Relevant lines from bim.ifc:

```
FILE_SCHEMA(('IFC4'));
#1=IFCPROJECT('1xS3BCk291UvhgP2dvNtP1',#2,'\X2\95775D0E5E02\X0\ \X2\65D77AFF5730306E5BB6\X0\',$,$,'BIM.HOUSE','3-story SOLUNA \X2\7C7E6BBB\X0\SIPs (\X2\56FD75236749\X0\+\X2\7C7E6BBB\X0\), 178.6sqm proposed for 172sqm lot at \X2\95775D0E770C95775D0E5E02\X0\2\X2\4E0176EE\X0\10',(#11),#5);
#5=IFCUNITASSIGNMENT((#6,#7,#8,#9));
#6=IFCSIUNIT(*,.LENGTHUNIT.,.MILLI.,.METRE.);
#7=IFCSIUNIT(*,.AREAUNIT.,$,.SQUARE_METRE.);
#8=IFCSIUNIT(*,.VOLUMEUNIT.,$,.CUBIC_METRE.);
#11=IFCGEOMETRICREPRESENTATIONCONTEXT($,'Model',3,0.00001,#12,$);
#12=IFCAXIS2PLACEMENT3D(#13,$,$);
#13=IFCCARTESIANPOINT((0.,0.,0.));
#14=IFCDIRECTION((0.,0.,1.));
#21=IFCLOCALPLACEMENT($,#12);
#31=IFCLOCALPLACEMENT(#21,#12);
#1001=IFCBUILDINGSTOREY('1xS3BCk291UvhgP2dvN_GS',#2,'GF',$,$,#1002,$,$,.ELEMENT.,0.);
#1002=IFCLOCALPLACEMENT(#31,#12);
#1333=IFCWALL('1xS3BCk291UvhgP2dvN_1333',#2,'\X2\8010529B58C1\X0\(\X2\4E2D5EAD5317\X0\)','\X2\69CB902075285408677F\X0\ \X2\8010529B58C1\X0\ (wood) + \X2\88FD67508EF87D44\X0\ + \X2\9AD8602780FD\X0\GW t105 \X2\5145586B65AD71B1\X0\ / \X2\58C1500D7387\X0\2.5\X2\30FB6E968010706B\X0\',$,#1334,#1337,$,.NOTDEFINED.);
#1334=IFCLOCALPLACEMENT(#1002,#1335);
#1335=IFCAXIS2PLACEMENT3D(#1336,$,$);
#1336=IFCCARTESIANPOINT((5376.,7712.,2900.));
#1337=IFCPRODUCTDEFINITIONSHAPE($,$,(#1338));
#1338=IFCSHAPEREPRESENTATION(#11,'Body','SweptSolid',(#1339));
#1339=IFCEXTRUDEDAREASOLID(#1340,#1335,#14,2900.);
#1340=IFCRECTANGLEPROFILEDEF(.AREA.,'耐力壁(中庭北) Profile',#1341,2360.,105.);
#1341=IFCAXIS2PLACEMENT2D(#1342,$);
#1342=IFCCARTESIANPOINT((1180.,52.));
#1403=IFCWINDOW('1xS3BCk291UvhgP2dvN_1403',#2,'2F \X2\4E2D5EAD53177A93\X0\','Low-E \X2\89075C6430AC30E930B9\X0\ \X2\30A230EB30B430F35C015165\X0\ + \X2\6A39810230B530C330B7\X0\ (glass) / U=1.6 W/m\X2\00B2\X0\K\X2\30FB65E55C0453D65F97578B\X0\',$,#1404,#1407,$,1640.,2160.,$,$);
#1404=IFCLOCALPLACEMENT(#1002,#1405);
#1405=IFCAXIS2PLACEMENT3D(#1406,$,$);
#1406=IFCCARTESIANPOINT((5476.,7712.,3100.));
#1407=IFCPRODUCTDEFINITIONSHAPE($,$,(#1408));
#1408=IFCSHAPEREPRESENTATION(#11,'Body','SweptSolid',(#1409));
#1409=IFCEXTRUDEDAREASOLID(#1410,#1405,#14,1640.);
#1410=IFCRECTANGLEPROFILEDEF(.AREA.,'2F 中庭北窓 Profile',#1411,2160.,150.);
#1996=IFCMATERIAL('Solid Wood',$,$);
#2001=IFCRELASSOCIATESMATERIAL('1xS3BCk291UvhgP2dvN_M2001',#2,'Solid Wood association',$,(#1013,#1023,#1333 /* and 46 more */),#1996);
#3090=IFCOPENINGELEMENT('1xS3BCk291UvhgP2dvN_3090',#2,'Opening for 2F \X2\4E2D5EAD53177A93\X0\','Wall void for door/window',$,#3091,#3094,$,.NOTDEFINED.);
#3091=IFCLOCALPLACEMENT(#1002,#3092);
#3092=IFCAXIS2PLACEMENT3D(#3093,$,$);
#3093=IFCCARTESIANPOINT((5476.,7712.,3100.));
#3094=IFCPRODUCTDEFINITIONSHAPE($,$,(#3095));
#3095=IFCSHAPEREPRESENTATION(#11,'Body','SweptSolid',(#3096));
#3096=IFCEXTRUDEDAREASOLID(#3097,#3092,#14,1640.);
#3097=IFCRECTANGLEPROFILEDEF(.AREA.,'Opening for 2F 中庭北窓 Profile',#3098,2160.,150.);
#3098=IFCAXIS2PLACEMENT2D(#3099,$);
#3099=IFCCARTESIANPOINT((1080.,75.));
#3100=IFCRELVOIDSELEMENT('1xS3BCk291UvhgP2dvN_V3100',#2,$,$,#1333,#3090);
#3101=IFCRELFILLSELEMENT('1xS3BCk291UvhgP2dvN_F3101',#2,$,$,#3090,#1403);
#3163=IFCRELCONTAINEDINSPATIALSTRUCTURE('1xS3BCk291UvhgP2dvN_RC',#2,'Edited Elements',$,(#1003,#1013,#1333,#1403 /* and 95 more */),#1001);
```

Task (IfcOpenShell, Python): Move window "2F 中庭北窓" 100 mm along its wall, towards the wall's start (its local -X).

```python
import ifcopenshell
import ifcopenshell.api.geometry
import ifcopenshell.util.placement

model = ifcopenshell.open("bim.ifc")

window = model.by_guid("1xS3BCk291UvhgP2dvN_1403")
opening = window.FillsVoids[0].RelatingOpeningElement
wall = opening.VoidsElements[0].RelatingBuildingElement

wall_matrix = ifcopenshell.util.placement.get_local_placement(wall.ObjectPlacement)
shift = wall_matrix[:3, 0] * -100.0
before = ifcopenshell.util.placement.get_local_placement(window.ObjectPlacement)[:3, 3].copy()

# The window is not placed relative to its opening, so move both.
for product in (opening, window):
    matrix = ifcopenshell.util.placement.get_local_placement(product.ObjectPlacement)
    matrix[:3, 3] += shift
    ifcopenshell.api.geometry.edit_object_placement(model, product=product, matrix=matrix, is_si=False)

after = ifcopenshell.util.placement.get_local_placement(window.ObjectPlacement)[:3, 3]
print("window moved by", (after - before).round(3) + 0.0)

model.write("bim_edited.ifc")
```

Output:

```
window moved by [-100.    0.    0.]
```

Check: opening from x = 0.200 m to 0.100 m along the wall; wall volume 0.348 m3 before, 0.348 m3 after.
